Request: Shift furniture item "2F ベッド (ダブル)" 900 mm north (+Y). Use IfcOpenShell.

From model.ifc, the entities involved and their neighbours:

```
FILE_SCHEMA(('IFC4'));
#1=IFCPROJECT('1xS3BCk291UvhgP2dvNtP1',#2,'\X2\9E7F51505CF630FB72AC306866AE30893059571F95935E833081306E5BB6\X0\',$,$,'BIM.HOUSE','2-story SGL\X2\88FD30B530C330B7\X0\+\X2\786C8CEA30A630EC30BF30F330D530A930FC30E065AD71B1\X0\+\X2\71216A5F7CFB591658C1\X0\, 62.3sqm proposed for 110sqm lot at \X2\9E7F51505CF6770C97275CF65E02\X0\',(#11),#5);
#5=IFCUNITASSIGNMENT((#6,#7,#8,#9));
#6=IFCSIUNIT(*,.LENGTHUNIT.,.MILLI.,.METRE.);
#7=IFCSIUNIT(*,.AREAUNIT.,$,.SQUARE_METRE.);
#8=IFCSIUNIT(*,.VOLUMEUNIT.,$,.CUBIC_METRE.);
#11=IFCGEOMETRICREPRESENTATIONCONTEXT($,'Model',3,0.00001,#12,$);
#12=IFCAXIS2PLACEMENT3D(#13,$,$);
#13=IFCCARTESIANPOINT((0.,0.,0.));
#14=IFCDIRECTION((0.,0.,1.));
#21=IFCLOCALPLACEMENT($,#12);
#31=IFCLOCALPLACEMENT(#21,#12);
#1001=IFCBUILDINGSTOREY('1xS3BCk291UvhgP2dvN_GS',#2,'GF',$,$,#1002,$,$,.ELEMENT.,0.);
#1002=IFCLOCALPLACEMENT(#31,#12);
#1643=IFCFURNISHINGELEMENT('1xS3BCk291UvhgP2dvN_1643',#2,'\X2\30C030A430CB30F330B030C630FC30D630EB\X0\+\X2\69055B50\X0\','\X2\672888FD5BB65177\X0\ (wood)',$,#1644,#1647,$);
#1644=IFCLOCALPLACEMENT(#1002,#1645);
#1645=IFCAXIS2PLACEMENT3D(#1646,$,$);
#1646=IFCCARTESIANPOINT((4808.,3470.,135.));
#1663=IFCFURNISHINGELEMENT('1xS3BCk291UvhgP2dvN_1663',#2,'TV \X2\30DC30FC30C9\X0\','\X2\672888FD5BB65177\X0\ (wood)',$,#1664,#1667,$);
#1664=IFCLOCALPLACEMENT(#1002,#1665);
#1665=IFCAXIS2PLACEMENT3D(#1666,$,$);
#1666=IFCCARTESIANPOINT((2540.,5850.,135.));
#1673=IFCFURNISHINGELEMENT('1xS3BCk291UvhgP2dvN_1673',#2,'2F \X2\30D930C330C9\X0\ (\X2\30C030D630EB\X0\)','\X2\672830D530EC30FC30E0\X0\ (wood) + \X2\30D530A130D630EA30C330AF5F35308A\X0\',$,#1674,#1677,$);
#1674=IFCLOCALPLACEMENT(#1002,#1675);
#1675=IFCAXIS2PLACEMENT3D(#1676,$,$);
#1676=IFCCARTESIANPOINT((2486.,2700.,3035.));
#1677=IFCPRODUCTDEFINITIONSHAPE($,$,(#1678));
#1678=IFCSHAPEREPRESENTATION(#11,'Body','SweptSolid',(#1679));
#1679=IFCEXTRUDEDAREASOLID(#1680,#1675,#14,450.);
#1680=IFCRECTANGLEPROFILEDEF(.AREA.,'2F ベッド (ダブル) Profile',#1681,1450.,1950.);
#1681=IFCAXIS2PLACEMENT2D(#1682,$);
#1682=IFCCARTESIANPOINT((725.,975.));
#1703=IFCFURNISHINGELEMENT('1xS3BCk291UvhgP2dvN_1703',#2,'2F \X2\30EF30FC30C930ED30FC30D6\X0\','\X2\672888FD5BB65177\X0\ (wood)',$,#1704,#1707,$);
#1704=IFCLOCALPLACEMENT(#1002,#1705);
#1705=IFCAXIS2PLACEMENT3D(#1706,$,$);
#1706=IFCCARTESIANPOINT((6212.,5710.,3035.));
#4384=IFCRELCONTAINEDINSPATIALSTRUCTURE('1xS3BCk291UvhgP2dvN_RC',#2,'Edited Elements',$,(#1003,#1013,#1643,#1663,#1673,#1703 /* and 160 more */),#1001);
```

```python
import ifcopenshell
import ifcopenshell.api.geometry
import ifcopenshell.util.placement
import ifcopenshell.util.unit

model = ifcopenshell.open("model.ifc")
unit_scale = ifcopenshell.util.unit.calculate_unit_scale(model)

item = model.by_id(1673)
matrix = ifcopenshell.util.placement.get_local_placement(item.ObjectPlacement)
matrix[1, 3] += 0.9 / unit_scale
ifcopenshell.api.geometry.edit_object_placement(model, product=item, matrix=matrix, is_si=False)

print(ifcopenshell.util.placement.get_local_placement(item.ObjectPlacement).round(3) + 0.0)

model.write("model_v2.ifc")
```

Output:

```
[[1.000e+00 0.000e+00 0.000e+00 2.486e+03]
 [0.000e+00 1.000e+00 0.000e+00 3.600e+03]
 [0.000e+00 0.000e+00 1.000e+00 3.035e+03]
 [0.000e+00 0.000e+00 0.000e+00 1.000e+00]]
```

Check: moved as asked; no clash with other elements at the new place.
